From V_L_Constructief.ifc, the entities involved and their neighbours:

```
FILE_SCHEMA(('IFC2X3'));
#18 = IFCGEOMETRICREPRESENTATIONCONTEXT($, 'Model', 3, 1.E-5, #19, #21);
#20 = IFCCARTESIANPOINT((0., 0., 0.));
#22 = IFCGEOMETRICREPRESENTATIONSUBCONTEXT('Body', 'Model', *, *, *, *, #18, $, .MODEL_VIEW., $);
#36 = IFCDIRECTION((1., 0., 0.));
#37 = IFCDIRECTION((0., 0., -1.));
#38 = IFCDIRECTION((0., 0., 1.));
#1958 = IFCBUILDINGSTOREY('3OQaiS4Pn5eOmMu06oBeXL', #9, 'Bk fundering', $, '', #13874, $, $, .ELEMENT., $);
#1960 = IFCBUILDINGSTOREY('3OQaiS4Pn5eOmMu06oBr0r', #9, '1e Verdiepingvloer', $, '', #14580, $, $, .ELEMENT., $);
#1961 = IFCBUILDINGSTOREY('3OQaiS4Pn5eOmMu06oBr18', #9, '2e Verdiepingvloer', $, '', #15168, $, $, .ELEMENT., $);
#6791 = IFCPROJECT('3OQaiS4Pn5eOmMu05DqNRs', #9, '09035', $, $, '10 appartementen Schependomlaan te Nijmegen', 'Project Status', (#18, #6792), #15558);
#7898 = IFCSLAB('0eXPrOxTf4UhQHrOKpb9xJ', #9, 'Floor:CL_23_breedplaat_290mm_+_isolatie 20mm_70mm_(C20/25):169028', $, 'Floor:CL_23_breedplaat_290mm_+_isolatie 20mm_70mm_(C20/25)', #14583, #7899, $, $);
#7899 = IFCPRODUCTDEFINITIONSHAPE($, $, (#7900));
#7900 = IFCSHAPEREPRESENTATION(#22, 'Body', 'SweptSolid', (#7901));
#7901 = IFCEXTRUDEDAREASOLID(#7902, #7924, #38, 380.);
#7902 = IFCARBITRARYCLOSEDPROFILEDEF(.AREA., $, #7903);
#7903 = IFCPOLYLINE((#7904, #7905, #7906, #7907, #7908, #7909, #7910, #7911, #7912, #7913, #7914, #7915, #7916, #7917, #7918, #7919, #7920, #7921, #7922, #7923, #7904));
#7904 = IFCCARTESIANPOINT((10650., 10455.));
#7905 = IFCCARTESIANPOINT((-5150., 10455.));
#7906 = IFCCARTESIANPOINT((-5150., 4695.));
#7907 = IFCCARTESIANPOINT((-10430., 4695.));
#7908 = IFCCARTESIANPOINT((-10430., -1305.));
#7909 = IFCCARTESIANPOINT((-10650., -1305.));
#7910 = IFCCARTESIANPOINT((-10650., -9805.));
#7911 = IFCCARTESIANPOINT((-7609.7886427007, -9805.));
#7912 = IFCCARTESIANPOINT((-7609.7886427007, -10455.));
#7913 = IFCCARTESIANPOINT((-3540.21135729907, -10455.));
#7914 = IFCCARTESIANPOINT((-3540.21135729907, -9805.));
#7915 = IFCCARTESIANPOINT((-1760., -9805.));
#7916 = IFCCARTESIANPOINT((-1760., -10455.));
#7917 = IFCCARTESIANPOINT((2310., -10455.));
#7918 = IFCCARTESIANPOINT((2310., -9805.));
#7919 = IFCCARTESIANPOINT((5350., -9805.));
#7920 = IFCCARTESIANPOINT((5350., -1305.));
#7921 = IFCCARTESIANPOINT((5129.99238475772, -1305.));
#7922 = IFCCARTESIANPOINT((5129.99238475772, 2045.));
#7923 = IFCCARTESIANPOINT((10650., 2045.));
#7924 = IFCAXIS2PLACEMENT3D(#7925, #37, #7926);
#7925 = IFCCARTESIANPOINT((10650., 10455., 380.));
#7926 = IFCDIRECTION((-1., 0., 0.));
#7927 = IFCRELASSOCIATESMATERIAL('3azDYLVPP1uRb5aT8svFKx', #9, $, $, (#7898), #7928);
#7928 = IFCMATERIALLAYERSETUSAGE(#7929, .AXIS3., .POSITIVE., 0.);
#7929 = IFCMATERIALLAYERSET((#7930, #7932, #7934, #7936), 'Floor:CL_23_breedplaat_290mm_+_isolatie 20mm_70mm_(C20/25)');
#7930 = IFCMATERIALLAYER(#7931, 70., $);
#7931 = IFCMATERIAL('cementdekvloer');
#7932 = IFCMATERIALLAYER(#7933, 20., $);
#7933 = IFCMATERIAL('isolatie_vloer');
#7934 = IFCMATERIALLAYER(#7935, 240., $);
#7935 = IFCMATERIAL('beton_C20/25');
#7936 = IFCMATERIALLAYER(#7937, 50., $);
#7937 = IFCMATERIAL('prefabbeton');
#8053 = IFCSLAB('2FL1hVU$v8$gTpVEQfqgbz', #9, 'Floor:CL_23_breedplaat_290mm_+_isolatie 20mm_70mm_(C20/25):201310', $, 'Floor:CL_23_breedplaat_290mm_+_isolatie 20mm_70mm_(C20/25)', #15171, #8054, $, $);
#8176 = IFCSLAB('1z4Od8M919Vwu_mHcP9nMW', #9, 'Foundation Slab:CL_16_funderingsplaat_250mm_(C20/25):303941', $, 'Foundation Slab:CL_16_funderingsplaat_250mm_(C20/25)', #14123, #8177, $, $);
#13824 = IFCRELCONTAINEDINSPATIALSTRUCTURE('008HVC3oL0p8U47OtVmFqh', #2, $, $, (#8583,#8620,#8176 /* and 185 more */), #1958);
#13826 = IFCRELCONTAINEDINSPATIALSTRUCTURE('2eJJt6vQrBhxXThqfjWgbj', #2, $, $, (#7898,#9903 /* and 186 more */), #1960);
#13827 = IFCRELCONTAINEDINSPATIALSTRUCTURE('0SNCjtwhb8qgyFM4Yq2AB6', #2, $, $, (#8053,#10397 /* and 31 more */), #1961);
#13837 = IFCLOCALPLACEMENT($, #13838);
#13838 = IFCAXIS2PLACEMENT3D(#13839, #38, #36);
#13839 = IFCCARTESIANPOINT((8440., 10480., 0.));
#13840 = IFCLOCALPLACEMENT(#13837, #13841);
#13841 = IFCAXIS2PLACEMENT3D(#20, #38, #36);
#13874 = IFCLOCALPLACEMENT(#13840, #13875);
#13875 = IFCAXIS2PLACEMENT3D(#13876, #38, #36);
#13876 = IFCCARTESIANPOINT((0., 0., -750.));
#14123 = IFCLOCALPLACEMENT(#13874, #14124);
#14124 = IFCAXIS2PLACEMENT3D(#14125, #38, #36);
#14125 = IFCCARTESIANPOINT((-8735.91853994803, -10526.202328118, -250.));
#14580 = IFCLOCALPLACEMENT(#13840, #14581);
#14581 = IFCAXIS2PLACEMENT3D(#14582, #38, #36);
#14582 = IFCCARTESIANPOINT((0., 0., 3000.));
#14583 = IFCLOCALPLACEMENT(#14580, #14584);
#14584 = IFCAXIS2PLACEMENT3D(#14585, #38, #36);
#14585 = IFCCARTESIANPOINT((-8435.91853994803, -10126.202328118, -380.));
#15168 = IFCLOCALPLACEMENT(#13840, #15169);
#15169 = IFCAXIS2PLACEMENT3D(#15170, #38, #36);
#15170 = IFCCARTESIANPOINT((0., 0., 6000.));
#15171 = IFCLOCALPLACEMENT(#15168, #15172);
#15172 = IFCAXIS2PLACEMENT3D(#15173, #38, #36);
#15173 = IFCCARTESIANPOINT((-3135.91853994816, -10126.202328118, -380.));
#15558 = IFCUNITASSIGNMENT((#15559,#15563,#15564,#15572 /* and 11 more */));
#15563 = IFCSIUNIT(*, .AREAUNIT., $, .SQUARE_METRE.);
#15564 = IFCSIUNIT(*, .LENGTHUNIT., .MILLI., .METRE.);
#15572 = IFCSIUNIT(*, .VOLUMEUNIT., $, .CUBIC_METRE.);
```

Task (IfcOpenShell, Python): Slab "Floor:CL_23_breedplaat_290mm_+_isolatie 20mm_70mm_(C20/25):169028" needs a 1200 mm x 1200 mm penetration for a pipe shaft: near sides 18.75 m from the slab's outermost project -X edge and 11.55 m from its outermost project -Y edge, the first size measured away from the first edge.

```python
import numpy as np
import ifcopenshell
import ifcopenshell.api.feature
import ifcopenshell.api.geometry
import ifcopenshell.api.root
import ifcopenshell.geom
import ifcopenshell.util.placement
import ifcopenshell.util.representation
import ifcopenshell.util.shape
import ifcopenshell.util.unit

model = ifcopenshell.open("V_L_Constructief.ifc")
unit_scale = ifcopenshell.util.unit.calculate_unit_scale(model)
settings = ifcopenshell.geom.settings()


def volume(element):
    """Net volume in cubic metres, openings subtracted."""
    shape = ifcopenshell.geom.create_shape(settings, element)
    return ifcopenshell.util.shape.get_volume(shape.geometry)


slab = model.by_id(7898)
before = volume(slab)

# Extent in the slab's own axes, in metres. The edges named are its -X and -Y sides.
slab_shape = ifcopenshell.geom.create_shape(settings, slab)
vertices = ifcopenshell.util.shape.get_vertices(slab_shape.geometry)
x_min, y_min, bottom = vertices.min(axis=0)
top = vertices[:, 2].max()

opening = ifcopenshell.api.root.create_entity(model, ifc_class="IfcOpeningElement", name="Pipe shaft opening")
context = ifcopenshell.util.representation.get_context(model, "Model", "Body", "MODEL_VIEW")
width, depth = 1.2, 1.2
outline = [(0.0, 0.0), (width, 0.0), (width, depth), (0.0, depth), (0.0, 0.0)]
# Overshoot both faces by 50 mm so the cut is clean.
shape = ifcopenshell.api.geometry.add_slab_representation(
    model, context=context, depth=top - bottom + 0.1, polyline=outline
)
ifcopenshell.api.geometry.assign_representation(model, product=opening, representation=shape)

matrix = ifcopenshell.util.placement.get_local_placement(slab.ObjectPlacement)
matrix[:, 3] = matrix @ np.append(np.array([x_min + 18.75, y_min + 11.55, bottom - 0.05]) / unit_scale, 1.0)
ifcopenshell.api.geometry.edit_object_placement(model, product=opening, matrix=matrix, is_si=False)
ifcopenshell.api.feature.add_feature(model, feature=opening, element=slab)

after = volume(slab)

print(f"slab volume {before:.3f} -> {after:.3f} m3")

model.write("V_L_Constructief_rev.ifc")
```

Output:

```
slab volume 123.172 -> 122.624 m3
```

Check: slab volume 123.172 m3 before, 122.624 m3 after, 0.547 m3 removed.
